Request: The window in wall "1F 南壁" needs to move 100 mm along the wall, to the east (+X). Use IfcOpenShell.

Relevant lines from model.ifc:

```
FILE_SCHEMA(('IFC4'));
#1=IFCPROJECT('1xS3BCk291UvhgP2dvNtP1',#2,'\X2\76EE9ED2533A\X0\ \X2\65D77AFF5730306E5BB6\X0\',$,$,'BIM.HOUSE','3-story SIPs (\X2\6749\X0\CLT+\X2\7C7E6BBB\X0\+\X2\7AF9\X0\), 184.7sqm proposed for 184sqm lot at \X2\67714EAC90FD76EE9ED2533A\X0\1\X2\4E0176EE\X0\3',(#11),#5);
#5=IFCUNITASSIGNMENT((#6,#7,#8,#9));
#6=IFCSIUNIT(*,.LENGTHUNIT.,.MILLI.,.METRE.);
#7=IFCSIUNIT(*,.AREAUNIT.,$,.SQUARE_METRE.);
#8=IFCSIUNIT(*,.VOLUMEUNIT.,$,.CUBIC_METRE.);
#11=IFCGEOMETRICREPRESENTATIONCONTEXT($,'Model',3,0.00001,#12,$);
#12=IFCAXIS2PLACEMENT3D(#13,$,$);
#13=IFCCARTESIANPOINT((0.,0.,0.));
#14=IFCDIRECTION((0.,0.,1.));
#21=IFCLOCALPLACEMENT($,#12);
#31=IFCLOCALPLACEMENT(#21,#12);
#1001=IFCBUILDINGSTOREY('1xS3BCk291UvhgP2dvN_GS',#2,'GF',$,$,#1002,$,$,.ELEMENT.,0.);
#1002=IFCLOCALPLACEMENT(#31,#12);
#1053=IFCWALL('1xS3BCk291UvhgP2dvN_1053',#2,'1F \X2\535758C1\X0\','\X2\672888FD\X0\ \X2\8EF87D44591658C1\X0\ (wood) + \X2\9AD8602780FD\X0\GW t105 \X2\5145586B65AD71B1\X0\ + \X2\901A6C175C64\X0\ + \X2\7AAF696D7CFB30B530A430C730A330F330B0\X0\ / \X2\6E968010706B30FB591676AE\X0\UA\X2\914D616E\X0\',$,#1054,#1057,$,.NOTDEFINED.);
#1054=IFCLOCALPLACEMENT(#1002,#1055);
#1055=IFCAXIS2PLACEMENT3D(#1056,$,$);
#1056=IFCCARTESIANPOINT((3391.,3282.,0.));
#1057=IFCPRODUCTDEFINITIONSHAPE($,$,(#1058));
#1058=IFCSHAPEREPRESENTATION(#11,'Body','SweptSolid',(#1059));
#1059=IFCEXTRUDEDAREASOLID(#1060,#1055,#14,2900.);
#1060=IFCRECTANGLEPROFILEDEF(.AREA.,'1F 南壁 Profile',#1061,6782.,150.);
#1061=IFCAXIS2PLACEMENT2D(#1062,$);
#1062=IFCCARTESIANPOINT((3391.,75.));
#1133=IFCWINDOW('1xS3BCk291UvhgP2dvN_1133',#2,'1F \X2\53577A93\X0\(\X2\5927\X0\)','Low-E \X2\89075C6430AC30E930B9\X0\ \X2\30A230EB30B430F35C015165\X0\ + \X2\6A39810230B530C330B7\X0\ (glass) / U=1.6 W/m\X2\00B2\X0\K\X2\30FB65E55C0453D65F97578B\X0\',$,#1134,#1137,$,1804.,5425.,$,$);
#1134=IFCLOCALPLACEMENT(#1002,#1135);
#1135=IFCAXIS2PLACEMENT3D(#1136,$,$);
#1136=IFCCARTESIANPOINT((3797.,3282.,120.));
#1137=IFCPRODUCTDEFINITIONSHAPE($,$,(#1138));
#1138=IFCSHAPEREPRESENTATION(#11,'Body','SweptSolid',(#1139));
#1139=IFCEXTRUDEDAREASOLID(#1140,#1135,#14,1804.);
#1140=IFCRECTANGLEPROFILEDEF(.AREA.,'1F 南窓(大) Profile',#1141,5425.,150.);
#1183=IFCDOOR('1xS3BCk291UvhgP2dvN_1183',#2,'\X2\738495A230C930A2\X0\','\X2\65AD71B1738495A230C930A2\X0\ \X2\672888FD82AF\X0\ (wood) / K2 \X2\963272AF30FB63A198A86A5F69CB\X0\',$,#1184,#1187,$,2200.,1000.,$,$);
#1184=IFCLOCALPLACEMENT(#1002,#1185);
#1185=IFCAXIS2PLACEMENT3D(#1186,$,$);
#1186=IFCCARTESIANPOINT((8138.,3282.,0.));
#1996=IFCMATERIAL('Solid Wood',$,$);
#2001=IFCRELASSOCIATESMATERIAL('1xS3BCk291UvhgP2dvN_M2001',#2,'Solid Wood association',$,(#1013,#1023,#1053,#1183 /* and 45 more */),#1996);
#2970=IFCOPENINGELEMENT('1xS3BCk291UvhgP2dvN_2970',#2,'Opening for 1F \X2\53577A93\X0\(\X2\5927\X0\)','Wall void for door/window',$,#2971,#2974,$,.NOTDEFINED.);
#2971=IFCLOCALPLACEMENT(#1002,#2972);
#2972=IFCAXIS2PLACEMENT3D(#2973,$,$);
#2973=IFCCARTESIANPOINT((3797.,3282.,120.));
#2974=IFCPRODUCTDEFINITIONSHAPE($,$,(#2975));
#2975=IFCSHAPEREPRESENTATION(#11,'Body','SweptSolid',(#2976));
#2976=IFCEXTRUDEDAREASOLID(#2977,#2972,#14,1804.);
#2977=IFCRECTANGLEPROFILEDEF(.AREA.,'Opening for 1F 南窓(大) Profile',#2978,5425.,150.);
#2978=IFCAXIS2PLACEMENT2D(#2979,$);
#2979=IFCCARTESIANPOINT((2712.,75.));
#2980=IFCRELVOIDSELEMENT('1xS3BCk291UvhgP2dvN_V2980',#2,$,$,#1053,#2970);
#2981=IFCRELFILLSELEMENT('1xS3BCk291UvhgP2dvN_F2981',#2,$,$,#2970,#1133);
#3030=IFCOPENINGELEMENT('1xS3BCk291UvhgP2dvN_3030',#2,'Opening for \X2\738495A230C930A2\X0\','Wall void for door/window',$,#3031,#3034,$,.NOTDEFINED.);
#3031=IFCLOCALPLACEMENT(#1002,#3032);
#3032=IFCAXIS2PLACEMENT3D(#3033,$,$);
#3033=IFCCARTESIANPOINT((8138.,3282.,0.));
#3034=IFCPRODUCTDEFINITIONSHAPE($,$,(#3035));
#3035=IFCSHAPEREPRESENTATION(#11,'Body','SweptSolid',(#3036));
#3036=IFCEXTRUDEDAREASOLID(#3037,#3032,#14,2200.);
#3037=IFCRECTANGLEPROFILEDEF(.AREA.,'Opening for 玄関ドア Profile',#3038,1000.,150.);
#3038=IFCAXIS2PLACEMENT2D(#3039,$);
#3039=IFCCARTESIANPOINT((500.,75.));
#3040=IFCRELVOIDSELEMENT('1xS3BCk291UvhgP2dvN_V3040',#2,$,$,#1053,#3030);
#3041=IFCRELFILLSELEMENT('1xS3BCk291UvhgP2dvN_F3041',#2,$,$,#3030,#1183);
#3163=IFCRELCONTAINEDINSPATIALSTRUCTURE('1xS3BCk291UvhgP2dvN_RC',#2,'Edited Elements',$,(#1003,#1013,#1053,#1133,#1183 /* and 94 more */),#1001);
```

```python
import ifcopenshell
import ifcopenshell.api.geometry
import ifcopenshell.util.placement
import ifcopenshell.util.unit

model = ifcopenshell.open("model.ifc")
unit_scale = ifcopenshell.util.unit.calculate_unit_scale(model)

window = model.by_guid("1xS3BCk291UvhgP2dvN_1133")
opening = window.FillsVoids[0].RelatingOpeningElement
wall = opening.VoidsElements[0].RelatingBuildingElement

wall_matrix = ifcopenshell.util.placement.get_local_placement(wall.ObjectPlacement)
shift = wall_matrix[:3, 0] * 0.1 / unit_scale
before = ifcopenshell.util.placement.get_local_placement(window.ObjectPlacement)[:3, 3].copy()

# The window is not placed relative to its opening, so move both.
for product in (opening, window):
    matrix = ifcopenshell.util.placement.get_local_placement(product.ObjectPlacement)
    matrix[:3, 3] += shift
    ifcopenshell.api.geometry.edit_object_placement(model, product=product, matrix=matrix, is_si=False)

after = ifcopenshell.util.placement.get_local_placement(window.ObjectPlacement)[:3, 3]
print("window moved by", (after - before).round(3) + 0.0)

model.write("model_rev.ifc")
```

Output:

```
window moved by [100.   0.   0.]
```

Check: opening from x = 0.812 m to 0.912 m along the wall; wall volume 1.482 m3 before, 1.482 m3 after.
